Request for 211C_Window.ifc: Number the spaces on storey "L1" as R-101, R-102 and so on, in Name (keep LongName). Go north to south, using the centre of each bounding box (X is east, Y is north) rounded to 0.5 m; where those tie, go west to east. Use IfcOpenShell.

First a look at what the model holds.

```python
import ifcopenshell
import ifcopenshell.util.element
import ifcopenshell.util.placement

model = ifcopenshell.open("211C_Window.ifc")
print(model.schema)
storey = next(s for s in model.by_type("IfcBuildingStorey") if s.Name == "L1")
spaces = [e for e in ifcopenshell.util.element.get_decomposition(storey) if e.is_a("IfcSpace")]
for e in sorted(spaces, key=lambda e: e.id()):
    origin = ifcopenshell.util.placement.get_local_placement(e.ObjectPlacement)[:3, 3]
    print(e.id(), e.Name, e.LongName, origin.round(2) + 0.0, sep=" | ")
```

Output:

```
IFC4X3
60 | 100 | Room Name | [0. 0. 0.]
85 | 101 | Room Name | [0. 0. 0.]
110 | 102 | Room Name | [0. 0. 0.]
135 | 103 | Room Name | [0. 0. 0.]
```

```python
import ifcopenshell
import ifcopenshell.geom
import ifcopenshell.util.element
import ifcopenshell.util.shape

model = ifcopenshell.open("211C_Window.ifc")
settings = ifcopenshell.geom.settings()
settings.set("use-world-coords", True)


def centre(element):
    shape = ifcopenshell.geom.create_shape(settings, element)
    return ifcopenshell.util.shape.get_bbox_centroid(shape.geometry)


storey = next(s for s in model.by_type("IfcBuildingStorey") if s.Name == "L1")
spaces = [e for e in ifcopenshell.util.element.get_decomposition(storey) if e.is_a("IfcSpace")]

# Insertion points can sit at a corner or the storey origin, so sort by the geometry (in metres).
centres = {e: centre(e) for e in spaces}
spaces.sort(key=lambda e: (-round(centres[e][1] / 0.5), centres[e][0]))

for i, e in enumerate(spaces, start=1):
    number = f"R-1{i:02d}"
    e.Name = number
    print(e.id(), number)

model.write("211C_Window_rev.ifc")
```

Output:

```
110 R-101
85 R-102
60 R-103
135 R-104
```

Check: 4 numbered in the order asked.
